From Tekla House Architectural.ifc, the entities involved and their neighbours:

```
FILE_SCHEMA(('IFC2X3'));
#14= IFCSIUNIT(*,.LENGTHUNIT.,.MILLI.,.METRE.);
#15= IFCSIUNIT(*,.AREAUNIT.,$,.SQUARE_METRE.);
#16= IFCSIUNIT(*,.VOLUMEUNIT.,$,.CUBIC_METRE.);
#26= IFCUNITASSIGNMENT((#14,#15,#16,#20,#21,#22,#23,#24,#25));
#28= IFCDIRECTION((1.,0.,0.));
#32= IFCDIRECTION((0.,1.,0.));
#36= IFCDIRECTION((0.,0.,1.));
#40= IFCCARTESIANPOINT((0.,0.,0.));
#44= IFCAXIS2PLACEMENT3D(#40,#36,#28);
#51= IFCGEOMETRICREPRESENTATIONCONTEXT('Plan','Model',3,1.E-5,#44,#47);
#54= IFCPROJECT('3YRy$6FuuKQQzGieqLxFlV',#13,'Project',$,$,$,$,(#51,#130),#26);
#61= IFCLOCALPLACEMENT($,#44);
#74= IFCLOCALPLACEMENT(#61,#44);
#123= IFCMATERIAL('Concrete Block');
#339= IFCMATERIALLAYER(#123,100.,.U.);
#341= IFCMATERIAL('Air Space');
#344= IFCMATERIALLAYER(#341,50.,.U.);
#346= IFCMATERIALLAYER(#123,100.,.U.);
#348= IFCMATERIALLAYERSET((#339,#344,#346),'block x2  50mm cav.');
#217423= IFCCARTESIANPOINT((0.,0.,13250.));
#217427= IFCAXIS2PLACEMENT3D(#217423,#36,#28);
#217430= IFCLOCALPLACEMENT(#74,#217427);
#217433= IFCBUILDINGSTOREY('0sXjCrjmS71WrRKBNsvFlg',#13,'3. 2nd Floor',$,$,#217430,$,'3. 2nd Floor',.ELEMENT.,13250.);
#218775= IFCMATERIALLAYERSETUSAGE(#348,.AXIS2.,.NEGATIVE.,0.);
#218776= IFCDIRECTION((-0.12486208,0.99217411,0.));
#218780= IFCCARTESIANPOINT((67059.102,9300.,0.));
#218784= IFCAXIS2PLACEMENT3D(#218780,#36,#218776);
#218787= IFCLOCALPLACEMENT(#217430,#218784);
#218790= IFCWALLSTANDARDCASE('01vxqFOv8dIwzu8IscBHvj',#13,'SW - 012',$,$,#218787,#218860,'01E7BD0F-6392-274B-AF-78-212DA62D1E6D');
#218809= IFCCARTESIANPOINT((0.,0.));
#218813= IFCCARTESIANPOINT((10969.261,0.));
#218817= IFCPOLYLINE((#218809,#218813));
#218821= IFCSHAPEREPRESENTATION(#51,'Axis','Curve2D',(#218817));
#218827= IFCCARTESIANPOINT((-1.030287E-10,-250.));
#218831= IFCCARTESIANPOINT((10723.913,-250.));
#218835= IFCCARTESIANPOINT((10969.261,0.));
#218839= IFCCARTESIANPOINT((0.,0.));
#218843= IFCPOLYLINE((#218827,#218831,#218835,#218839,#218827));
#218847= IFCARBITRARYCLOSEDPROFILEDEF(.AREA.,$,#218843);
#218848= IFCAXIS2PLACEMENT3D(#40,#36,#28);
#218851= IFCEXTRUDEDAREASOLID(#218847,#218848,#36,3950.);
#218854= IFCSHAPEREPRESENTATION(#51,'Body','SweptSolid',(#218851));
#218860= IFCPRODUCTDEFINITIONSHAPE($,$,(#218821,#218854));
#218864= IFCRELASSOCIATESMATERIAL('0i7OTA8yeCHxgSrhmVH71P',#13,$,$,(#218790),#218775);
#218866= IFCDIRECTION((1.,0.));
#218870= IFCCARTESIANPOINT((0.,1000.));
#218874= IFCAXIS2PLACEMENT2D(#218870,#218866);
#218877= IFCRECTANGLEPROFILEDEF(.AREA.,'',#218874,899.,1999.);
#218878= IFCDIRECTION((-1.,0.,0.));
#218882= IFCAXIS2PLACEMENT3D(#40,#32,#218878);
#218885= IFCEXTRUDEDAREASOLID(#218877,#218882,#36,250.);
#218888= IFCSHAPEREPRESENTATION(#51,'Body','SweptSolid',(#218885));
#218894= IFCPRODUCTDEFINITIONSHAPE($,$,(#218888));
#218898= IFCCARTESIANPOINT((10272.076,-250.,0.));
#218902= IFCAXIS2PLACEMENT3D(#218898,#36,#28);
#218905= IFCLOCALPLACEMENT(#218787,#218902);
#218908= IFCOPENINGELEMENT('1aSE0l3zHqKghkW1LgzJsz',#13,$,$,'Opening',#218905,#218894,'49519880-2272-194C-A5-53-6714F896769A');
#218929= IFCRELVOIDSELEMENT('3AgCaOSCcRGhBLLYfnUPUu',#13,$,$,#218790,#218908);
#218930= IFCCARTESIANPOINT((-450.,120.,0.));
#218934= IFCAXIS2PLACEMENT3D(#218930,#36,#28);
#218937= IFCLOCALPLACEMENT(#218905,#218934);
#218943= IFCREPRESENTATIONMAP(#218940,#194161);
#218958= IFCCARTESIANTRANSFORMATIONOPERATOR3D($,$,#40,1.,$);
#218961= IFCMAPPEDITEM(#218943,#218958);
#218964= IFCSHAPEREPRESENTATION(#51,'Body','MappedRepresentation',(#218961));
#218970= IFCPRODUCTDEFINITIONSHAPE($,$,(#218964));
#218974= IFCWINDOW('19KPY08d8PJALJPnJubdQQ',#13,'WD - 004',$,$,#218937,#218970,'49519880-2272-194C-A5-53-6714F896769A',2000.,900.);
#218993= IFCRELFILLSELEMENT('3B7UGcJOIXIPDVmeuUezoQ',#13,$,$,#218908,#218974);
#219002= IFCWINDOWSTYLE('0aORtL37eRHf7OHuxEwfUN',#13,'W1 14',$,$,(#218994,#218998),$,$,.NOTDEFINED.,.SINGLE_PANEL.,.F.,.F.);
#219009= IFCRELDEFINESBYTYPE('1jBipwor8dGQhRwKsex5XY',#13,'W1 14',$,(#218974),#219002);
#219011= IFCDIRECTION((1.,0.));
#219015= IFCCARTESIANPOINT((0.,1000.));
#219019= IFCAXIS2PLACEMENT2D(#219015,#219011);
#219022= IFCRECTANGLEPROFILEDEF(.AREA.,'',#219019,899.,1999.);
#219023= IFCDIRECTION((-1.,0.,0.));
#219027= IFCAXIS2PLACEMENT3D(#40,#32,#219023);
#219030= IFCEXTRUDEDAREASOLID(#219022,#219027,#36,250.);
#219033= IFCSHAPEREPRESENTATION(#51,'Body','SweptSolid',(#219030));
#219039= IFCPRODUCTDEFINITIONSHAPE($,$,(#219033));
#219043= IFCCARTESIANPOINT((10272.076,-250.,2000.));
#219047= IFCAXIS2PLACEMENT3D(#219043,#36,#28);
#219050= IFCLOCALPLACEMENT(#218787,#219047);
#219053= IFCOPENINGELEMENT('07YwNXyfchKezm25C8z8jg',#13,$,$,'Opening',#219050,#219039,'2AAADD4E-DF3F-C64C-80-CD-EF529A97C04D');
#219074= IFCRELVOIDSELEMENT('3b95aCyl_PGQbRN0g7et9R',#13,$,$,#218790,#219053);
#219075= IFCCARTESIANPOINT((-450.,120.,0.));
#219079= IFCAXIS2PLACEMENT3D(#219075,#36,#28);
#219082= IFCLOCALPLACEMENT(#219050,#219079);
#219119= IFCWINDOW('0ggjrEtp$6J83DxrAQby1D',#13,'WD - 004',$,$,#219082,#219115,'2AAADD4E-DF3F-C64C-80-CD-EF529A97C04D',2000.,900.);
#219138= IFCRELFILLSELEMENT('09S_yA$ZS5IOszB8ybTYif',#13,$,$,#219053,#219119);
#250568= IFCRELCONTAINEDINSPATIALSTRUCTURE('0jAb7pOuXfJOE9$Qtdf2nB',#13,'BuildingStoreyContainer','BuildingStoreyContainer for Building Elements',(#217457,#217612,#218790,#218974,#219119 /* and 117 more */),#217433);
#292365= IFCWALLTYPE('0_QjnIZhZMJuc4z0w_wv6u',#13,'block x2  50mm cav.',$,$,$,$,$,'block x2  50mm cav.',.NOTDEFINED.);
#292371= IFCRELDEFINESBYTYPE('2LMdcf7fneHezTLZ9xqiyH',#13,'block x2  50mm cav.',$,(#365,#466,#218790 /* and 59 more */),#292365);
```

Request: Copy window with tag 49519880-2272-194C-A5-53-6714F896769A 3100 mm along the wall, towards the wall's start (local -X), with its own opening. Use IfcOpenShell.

```python
import ifcopenshell
import ifcopenshell.api.feature
import ifcopenshell.api.geometry
import ifcopenshell.api.root
import ifcopenshell.geom
import ifcopenshell.util.element
import ifcopenshell.util.placement
import ifcopenshell.util.shape
import ifcopenshell.util.unit

model = ifcopenshell.open("Tekla House Architectural.ifc")
unit_scale = ifcopenshell.util.unit.calculate_unit_scale(model)
settings = ifcopenshell.geom.settings()


def volume(element):
    """Net volume in cubic metres, openings subtracted."""
    shape = ifcopenshell.geom.create_shape(settings, element)
    return ifcopenshell.util.shape.get_volume(shape.geometry)


window = model.by_guid("19KPY08d8PJALJPnJubdQQ")
opening = window.FillsVoids[0].RelatingOpeningElement
wall = opening.VoidsElements[0].RelatingBuildingElement
before = volume(wall)
shift = ifcopenshell.util.placement.get_local_placement(wall.ObjectPlacement)[:3, 0] * -3.1 / unit_scale

# copy_class copies the void relationship, type, container and properties, but no geometry.
new_opening = ifcopenshell.api.root.copy_class(model, product=opening)
new_opening.Representation = ifcopenshell.util.element.copy_deep(
    model, opening.Representation, exclude=["IfcGeometricRepresentationContext", "IfcRepresentationMap"]
)
new_opening.Tag = None
new_window = ifcopenshell.api.root.copy_class(model, product=window)
new_window.Representation = ifcopenshell.util.element.copy_deep(
    model, window.Representation, exclude=["IfcGeometricRepresentationContext", "IfcRepresentationMap"]
)
new_window.Tag = None
fills = ifcopenshell.api.feature.add_filling(model, opening=new_opening, element=new_window)
fills.OwnerHistory = new_window.OwnerHistory  # required in IFC2X3

for old, new in ((opening, new_opening), (window, new_window)):
    matrix = ifcopenshell.util.placement.get_local_placement(old.ObjectPlacement)
    matrix[:3, 3] += shift
    ifcopenshell.api.geometry.edit_object_placement(model, product=new, matrix=matrix, is_si=False)

after = volume(wall)

print(f"wall volume {before:.3f} -> {after:.3f} m3")

model.write("Tekla House Architectural_edited.ifc")
```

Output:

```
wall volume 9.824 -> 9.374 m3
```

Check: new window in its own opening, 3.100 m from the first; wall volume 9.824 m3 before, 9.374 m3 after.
